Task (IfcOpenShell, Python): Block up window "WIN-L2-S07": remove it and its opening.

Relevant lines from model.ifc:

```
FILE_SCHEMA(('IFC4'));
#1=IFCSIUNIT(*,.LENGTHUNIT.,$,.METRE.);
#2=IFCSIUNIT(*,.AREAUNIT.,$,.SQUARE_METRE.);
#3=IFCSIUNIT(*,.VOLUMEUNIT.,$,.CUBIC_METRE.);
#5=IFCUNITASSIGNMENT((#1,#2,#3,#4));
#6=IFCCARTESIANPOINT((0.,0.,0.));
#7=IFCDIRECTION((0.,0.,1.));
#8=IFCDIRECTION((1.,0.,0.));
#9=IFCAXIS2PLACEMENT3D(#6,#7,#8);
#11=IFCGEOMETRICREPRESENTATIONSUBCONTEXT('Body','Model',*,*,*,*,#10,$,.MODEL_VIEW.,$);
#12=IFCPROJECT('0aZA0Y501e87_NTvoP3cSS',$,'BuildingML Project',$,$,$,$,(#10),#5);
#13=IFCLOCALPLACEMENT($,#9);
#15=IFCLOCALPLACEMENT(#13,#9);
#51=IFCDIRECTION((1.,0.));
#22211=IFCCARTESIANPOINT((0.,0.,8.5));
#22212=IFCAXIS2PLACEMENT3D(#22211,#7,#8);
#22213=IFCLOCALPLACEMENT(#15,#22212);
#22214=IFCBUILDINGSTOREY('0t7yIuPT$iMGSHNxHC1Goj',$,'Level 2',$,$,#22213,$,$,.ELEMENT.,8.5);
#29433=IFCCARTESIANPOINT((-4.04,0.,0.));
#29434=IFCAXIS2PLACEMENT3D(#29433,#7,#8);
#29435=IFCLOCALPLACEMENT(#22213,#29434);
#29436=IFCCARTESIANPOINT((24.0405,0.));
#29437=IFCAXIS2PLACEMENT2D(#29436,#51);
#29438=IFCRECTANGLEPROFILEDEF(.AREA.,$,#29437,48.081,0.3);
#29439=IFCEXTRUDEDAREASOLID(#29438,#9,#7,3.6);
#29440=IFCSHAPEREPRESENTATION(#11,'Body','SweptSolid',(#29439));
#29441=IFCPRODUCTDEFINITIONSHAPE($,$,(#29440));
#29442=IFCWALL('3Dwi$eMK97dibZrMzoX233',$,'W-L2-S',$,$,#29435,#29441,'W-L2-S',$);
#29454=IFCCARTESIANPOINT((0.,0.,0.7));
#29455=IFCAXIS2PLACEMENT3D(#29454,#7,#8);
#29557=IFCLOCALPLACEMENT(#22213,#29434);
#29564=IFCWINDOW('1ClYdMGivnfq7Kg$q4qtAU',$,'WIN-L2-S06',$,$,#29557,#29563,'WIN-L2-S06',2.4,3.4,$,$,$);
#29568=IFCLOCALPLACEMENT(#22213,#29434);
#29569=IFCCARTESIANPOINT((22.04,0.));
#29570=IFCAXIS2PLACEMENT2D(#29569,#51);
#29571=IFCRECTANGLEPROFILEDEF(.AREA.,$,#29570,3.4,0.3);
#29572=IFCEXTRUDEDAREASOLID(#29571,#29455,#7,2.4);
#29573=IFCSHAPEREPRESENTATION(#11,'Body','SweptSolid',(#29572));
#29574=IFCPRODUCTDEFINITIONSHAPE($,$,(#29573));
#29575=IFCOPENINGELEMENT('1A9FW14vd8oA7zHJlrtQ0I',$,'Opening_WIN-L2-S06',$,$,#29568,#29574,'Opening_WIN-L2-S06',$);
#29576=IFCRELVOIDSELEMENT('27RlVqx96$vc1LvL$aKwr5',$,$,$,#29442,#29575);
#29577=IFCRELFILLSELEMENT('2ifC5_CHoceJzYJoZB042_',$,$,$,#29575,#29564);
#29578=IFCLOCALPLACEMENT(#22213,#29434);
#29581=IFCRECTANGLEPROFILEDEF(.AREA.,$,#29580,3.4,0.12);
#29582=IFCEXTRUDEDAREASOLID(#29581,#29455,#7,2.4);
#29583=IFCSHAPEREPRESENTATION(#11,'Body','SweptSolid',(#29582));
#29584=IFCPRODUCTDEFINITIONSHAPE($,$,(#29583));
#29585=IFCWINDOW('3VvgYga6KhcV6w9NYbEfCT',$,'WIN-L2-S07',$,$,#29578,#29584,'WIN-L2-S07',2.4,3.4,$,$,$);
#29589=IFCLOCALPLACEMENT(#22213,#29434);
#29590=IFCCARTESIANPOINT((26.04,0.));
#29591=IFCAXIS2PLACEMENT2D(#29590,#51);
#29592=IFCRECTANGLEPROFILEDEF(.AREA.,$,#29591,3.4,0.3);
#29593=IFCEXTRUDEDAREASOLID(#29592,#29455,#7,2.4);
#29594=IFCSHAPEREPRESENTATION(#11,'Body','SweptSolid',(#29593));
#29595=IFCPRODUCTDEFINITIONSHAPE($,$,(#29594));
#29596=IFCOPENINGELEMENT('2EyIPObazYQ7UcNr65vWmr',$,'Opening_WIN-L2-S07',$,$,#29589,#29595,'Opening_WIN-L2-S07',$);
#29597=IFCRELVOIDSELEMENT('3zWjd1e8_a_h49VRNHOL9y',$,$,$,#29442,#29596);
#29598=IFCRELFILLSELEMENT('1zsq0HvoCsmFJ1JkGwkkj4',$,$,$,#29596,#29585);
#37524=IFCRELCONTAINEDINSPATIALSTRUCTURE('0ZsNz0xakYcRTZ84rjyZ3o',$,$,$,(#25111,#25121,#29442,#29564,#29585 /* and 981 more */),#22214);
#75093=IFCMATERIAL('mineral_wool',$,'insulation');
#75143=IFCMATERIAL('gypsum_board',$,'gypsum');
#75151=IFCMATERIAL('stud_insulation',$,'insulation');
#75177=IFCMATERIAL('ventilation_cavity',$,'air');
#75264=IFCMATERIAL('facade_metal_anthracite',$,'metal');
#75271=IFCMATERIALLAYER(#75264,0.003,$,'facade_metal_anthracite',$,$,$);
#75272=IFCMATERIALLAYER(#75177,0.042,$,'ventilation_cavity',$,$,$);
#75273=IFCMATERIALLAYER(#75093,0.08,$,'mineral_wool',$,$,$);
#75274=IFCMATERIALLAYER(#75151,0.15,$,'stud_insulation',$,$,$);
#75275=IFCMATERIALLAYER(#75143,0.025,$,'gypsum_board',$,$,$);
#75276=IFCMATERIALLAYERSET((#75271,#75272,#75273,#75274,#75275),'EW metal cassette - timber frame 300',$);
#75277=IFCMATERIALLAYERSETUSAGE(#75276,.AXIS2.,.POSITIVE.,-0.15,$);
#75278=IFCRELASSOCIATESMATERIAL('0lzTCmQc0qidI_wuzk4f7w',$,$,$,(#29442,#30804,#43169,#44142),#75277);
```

```python
import ifcopenshell
import ifcopenshell.api.feature
import ifcopenshell.api.root
import ifcopenshell.geom
import ifcopenshell.util.shape

model = ifcopenshell.open("model.ifc")
settings = ifcopenshell.geom.settings()


def volume(element):
    """Net volume in cubic metres, openings subtracted."""
    shape = ifcopenshell.geom.create_shape(settings, element)
    return ifcopenshell.util.shape.get_volume(shape.geometry)


window = model.by_id(29585)
opening = window.FillsVoids[0].RelatingOpeningElement
wall = opening.VoidsElements[0].RelatingBuildingElement
before = volume(wall)

ifcopenshell.api.root.remove_product(model, product=window)
ifcopenshell.api.feature.remove_feature(model, feature=opening)

after = volume(wall)

print(f"wall volume {before:.3f} -> {after:.3f} m3")

model.write("model_updated.ifc")
```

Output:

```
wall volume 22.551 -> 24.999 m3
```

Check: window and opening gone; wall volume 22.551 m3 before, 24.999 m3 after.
